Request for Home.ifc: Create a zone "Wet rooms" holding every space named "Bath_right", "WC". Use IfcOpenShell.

First a look at what the model holds.

```python
import ifcopenshell

model = ifcopenshell.open("Home.ifc")
print(model.schema)
seen = {}
for space in model.by_type("IfcSpace"):
    seen[space.LongName] = seen.get(space.LongName, 0) + 1
for name, count in sorted(seen.items(), key=str):
    print(count, "x", name)
print("zones:", [z.Name for z in model.by_type("IfcZone")][:20])
```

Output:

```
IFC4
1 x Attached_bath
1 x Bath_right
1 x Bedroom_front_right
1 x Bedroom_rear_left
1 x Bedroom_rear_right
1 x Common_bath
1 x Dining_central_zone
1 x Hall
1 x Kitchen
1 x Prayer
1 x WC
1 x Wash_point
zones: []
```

```python
import ifcopenshell
import ifcopenshell.api.group
import ifcopenshell.api.root

model = ifcopenshell.open("Home.ifc")

names = {"Bath_right", "WC"}
spaces = [s for s in model.by_type("IfcSpace") if s.LongName in names]

zone = ifcopenshell.api.root.create_entity(model, ifc_class="IfcZone", name="Wet rooms")
ifcopenshell.api.group.assign_group(model, products=spaces, group=zone)
print(len(spaces), "spaces in", zone.Name)

model.write("Home_edited.ifc")
```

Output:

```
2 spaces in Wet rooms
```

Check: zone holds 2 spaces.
